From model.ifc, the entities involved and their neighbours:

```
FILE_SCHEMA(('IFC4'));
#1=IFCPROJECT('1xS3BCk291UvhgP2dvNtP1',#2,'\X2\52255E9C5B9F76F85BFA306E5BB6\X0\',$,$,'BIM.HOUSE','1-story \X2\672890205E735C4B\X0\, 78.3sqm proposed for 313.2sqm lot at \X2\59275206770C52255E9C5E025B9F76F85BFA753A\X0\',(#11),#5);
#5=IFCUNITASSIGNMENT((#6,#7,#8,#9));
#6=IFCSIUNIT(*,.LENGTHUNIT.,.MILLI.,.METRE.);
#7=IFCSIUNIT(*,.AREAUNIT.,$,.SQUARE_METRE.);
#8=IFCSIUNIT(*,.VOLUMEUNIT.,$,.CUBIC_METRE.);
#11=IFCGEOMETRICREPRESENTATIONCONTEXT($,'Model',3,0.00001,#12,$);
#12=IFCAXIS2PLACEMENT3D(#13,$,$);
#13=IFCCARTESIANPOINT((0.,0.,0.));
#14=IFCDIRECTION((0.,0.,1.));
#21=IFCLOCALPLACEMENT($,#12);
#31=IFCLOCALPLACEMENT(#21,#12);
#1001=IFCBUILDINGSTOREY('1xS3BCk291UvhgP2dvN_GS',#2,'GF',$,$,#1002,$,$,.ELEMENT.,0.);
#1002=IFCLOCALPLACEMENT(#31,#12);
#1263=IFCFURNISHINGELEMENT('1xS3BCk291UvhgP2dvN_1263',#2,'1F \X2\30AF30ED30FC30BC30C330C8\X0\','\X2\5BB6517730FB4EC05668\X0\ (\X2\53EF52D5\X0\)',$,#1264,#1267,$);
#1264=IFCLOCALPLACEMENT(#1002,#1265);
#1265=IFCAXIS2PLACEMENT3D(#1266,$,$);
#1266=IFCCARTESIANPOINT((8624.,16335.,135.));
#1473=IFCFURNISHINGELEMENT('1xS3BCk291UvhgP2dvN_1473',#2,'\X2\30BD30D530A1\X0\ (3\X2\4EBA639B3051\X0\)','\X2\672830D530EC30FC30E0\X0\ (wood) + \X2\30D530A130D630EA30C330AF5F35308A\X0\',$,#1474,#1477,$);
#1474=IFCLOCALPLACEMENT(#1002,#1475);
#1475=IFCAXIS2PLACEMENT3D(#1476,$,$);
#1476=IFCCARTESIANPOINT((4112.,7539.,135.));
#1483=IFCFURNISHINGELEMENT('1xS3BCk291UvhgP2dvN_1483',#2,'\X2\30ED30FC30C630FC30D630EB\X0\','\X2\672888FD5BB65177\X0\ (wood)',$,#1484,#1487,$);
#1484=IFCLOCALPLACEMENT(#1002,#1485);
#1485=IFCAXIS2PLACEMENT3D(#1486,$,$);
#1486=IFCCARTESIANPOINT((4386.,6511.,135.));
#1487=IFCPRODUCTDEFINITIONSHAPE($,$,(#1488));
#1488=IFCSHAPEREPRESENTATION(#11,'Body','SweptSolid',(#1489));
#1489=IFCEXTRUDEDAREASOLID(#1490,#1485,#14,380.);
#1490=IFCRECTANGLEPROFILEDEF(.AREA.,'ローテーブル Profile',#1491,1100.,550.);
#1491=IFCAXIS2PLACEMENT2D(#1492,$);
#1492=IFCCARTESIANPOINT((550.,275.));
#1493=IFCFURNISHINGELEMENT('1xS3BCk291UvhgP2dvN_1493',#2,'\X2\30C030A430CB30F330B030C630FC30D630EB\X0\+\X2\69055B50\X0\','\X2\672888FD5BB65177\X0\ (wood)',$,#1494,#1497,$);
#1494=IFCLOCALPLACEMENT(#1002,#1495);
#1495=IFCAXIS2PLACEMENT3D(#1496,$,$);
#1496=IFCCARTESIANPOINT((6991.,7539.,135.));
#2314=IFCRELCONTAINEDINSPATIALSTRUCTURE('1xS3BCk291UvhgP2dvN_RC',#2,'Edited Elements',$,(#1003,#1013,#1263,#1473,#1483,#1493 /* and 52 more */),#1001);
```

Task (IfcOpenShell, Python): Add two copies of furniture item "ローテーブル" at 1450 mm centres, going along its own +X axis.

```python
import ifcopenshell
import ifcopenshell.api.geometry
import ifcopenshell.api.root
import ifcopenshell.util.element
import ifcopenshell.util.placement
import ifcopenshell.util.unit

model = ifcopenshell.open("model.ifc")
unit_scale = ifcopenshell.util.unit.calculate_unit_scale(model)


def reuse_history(source, copy):
    """copy_class also copies each property set's owner history, people and application; keep the originals."""
    for rel in copy.IsDefinedBy:
        if rel.is_a("IfcRelDefinesByProperties") and (history := rel.RelatingPropertyDefinition.OwnerHistory):
            rel.RelatingPropertyDefinition.OwnerHistory = source.OwnerHistory
            ifcopenshell.util.element.remove_deep2(model, history)


source = model.by_guid("1xS3BCk291UvhgP2dvN_1483")
base = ifcopenshell.util.placement.get_local_placement(source.ObjectPlacement)
step = base[:3, 0] * 1.45 / unit_scale

for i in range(1, 3):
    copy = ifcopenshell.api.root.copy_class(model, product=source)
    copy.Representation = ifcopenshell.util.element.copy_deep(
        model, source.Representation, exclude=["IfcGeometricRepresentationContext", "IfcRepresentationMap"]
    )
    reuse_history(source, copy)
    matrix = base.copy()
    matrix[:3, 3] += i * step
    print("added at", matrix[:3, 3].round(3) + 0.0)
    ifcopenshell.api.geometry.edit_object_placement(model, product=copy, matrix=matrix, is_si=False)

model.write("model-out.ifc")
```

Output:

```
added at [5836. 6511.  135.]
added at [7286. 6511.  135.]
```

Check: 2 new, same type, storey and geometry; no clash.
